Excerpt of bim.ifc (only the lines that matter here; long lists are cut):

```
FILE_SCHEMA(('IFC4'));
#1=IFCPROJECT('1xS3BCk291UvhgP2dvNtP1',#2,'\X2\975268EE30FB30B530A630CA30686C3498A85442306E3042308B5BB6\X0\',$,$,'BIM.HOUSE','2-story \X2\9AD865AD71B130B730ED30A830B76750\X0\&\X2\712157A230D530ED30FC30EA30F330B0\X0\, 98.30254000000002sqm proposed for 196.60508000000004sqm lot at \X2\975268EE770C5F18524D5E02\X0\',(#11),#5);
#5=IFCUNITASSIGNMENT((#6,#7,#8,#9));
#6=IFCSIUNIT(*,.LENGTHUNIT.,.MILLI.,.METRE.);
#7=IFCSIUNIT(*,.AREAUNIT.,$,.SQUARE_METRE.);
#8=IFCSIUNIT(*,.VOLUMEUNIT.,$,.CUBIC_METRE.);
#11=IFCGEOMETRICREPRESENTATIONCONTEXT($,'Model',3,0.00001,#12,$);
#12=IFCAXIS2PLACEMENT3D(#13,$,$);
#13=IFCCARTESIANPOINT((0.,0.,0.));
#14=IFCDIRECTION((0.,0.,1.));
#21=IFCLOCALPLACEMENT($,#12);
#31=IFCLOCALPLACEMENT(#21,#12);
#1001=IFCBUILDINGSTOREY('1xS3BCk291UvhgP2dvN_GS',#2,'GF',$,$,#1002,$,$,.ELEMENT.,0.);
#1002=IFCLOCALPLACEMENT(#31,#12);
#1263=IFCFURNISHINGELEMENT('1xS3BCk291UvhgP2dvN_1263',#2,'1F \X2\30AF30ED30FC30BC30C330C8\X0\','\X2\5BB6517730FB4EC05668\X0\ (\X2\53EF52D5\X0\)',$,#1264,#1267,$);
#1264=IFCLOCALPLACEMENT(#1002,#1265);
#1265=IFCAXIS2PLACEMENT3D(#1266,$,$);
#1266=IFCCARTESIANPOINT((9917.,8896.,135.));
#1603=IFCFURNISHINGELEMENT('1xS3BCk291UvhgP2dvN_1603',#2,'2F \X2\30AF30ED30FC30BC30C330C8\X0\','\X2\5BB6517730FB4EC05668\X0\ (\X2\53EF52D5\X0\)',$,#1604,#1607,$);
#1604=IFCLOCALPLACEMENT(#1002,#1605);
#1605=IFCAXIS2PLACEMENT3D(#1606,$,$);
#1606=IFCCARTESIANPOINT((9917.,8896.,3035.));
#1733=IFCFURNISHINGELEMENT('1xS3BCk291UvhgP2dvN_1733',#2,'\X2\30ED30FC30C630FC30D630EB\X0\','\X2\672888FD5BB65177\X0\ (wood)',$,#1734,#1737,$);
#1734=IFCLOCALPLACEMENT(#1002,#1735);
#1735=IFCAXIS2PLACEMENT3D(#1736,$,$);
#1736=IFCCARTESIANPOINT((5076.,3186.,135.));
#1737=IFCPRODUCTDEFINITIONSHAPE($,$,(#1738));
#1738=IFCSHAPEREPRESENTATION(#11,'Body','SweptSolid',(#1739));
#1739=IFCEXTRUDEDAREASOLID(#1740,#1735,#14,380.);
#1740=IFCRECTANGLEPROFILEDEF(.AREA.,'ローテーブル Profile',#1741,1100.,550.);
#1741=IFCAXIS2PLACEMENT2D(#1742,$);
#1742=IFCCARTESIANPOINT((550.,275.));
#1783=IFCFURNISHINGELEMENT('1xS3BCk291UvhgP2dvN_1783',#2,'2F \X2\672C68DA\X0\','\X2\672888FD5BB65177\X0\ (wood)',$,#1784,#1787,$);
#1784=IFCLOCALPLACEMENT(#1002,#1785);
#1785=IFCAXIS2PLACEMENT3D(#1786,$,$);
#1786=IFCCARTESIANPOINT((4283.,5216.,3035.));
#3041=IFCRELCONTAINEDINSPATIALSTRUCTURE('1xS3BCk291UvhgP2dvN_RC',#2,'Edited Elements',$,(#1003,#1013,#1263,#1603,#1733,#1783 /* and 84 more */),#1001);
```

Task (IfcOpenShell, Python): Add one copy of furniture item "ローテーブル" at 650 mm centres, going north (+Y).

```python
import numpy as np
import ifcopenshell
import ifcopenshell.api.geometry
import ifcopenshell.api.root
import ifcopenshell.util.element
import ifcopenshell.util.placement

model = ifcopenshell.open("bim.ifc")


def reuse_history(source, copy):
    """copy_class also copies each property set's owner history, people and application; keep the originals."""
    for rel in copy.IsDefinedBy:
        if rel.is_a("IfcRelDefinesByProperties") and (history := rel.RelatingPropertyDefinition.OwnerHistory):
            rel.RelatingPropertyDefinition.OwnerHistory = source.OwnerHistory
            ifcopenshell.util.element.remove_deep2(model, history)


source = model.by_guid("1xS3BCk291UvhgP2dvN_1733")
base = ifcopenshell.util.placement.get_local_placement(source.ObjectPlacement)
step = np.array([0.0, 1.0, 0.0]) * 650.0

for i in range(1, 2):
    copy = ifcopenshell.api.root.copy_class(model, product=source)
    copy.Representation = ifcopenshell.util.element.copy_deep(
        model, source.Representation, exclude=["IfcGeometricRepresentationContext", "IfcRepresentationMap"]
    )
    reuse_history(source, copy)
    matrix = base.copy()
    matrix[:3, 3] += i * step
    print("added at", matrix[:3, 3].round(3) + 0.0)
    ifcopenshell.api.geometry.edit_object_placement(model, product=copy, matrix=matrix, is_si=False)

model.write("bim_edited.ifc")
```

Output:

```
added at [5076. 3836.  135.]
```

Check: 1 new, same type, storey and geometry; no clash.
